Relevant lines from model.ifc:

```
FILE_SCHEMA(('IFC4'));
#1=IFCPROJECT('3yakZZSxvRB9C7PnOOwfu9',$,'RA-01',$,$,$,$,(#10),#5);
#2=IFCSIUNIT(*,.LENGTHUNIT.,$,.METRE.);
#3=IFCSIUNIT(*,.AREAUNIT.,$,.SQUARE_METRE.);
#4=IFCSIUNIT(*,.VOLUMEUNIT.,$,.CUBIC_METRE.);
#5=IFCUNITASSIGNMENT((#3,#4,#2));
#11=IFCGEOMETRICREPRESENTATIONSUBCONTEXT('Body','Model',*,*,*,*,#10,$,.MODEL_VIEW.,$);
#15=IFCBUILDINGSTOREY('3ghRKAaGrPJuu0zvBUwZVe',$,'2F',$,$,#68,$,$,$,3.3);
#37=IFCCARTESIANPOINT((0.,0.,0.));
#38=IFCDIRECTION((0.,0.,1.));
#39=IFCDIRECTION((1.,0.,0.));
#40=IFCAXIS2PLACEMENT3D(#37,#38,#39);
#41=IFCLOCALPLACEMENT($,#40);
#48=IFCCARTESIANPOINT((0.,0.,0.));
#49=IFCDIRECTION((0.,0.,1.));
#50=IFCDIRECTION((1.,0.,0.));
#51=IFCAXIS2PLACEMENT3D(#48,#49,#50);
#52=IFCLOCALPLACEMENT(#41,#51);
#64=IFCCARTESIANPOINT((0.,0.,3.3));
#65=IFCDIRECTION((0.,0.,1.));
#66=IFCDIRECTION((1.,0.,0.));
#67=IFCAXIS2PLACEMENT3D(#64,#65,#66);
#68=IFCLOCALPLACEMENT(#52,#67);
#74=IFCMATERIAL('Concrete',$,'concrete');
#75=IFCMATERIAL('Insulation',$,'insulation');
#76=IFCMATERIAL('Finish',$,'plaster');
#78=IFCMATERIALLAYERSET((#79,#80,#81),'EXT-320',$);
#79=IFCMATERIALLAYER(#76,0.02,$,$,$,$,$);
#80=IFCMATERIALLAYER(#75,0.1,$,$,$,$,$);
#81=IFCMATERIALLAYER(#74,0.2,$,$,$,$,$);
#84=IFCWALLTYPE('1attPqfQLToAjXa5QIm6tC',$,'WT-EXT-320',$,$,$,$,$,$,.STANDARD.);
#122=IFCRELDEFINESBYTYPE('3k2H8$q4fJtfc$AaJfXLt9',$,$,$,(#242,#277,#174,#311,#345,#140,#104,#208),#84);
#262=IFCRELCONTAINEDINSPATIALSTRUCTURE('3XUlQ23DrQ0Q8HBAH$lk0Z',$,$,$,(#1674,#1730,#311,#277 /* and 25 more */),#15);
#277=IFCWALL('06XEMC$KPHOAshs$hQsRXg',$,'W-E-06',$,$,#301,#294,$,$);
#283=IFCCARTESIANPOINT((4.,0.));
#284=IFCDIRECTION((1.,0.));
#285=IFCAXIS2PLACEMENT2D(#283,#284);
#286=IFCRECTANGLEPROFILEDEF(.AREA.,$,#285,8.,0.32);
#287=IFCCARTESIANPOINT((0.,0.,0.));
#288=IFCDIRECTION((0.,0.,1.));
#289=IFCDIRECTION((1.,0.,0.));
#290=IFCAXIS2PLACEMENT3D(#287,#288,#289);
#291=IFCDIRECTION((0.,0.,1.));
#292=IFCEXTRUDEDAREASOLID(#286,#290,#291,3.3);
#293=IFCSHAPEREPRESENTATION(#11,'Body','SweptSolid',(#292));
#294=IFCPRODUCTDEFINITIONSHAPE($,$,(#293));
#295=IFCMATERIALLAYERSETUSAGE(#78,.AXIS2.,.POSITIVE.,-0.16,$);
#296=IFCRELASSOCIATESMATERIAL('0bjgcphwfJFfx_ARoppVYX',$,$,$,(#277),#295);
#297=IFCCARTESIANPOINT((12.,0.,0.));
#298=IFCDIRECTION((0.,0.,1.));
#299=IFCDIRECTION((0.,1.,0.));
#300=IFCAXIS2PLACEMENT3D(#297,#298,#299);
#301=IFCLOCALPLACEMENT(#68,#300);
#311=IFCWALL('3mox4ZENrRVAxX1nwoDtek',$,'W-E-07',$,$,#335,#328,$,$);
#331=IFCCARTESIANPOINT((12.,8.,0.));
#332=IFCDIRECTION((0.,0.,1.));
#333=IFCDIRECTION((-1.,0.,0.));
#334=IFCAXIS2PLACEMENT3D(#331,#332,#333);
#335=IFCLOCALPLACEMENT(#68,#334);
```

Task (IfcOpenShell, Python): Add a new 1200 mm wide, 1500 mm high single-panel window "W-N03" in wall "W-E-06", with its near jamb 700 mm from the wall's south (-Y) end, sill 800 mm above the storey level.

```python
import numpy as np
import ifcopenshell
import ifcopenshell.api.feature
import ifcopenshell.api.geometry
import ifcopenshell.api.root
import ifcopenshell.api.spatial
import ifcopenshell.geom
import ifcopenshell.util.element
import ifcopenshell.util.placement
import ifcopenshell.util.representation
import ifcopenshell.util.shape
import ifcopenshell.util.unit

model = ifcopenshell.open("model.ifc")
unit_scale = ifcopenshell.util.unit.calculate_unit_scale(model)
settings = ifcopenshell.geom.settings()


def volume(element):
    """Net volume in cubic metres, openings subtracted."""
    shape = ifcopenshell.geom.create_shape(settings, element)
    return ifcopenshell.util.shape.get_volume(shape.geometry)


wall = model.by_guid("06XEMC$KPHOAshs$hQsRXg")
storey = ifcopenshell.util.element.get_container(wall, ifc_class="IfcBuildingStorey")
context = ifcopenshell.util.representation.get_context(model, "Model", "Body", "MODEL_VIEW")
before = volume(wall)

width, height, from_end, sill = 1.2, 1.5, 0.7, 0.8  # metres

# The wall runs along its own X axis, and the end named is its -X end.
wall_shape = ifcopenshell.geom.create_shape(settings, wall)
x, y, z = ifcopenshell.util.shape.get_vertices(wall_shape.geometry).T
start = x.min() + from_end
face, thickness = float(y.min()), float(y.max() - y.min())
wall_matrix = ifcopenshell.util.placement.get_local_placement(wall.ObjectPlacement)
level = ifcopenshell.util.placement.get_local_placement(storey.ObjectPlacement)[2, 3]


def in_wall(x, y):
    """Placement at x, y metres in the wall's axes, at sill height."""
    matrix = wall_matrix.copy()
    matrix[:, 3] = wall_matrix @ np.array([x / unit_scale, y / unit_scale, 0.0, 1.0])
    matrix[2, 3] = level + sill / unit_scale
    return matrix


# Opening: a box that overshoots both wall faces by 50 mm.
opening = ifcopenshell.api.root.create_entity(model, ifc_class="IfcOpeningElement", predefined_type="OPENING")
box = ifcopenshell.api.geometry.add_wall_representation(
    model, context=context, length=width, height=height, thickness=thickness + 0.1
)
ifcopenshell.api.geometry.assign_representation(model, product=opening, representation=box)
ifcopenshell.api.geometry.edit_object_placement(model, product=opening, matrix=in_wall(start, face - 0.05), is_si=False)
ifcopenshell.api.feature.add_feature(model, feature=opening, element=wall)

window = ifcopenshell.api.root.create_entity(model, ifc_class="IfcWindow", name="W-N03", predefined_type="WINDOW")
window.OverallWidth, window.OverallHeight = width / unit_scale, height / unit_scale
window.PartitioningType = "SINGLE_PANEL"
body = ifcopenshell.api.geometry.add_window_representation(
    model,
    context=context,
    overall_width=window.OverallWidth,
    overall_height=window.OverallHeight,
    partition_type="SINGLE_PANEL",
)
ifcopenshell.api.geometry.assign_representation(model, product=window, representation=body)
ifcopenshell.api.spatial.assign_container(model, products=[window], relating_structure=storey)
ifcopenshell.api.feature.add_filling(model, opening=opening, element=window)

# Centre the window in the wall's thickness.
ifcopenshell.api.geometry.edit_object_placement(model, product=window, matrix=in_wall(start, face), is_si=False)
window_shape = ifcopenshell.geom.create_shape(settings, window)
depth = ifcopenshell.util.shape.get_vertices(window_shape.geometry)[:, 1]
offset = face + thickness / 2 - (depth.min() + depth.max()) / 2
ifcopenshell.api.geometry.edit_object_placement(model, product=window, matrix=in_wall(start, offset), is_si=False)

after = volume(wall)

print(f"wall volume {before:.3f} -> {after:.3f} m3")

model.write("model-out.ifc")
```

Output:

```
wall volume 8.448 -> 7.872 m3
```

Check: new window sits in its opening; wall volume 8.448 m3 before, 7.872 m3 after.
